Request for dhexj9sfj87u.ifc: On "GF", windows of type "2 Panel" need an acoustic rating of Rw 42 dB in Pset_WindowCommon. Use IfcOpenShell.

First a look at what the model holds.

```python
import ifcopenshell
import ifcopenshell.util.element

model = ifcopenshell.open("dhexj9sfj87u.ifc")
print(model.schema)
storey = next(s for s in model.by_type("IfcBuildingStorey") if s.Name == "GF")
windows = [e for e in ifcopenshell.util.element.get_decomposition(storey) if e.is_a("IfcWindow")]
seen = {}
for e in windows:
    element_type = ifcopenshell.util.element.get_type(e)
    key = (element_type.Name if element_type != e and element_type else None, ifcopenshell.util.element.get_pset(e, "Pset_WindowCommon", "AcousticRating"))
    seen[key] = seen.get(key, 0) + 1
for (name, value), count in sorted(seen.items(), key=str):
    print(count, "x", name, "|", value)
```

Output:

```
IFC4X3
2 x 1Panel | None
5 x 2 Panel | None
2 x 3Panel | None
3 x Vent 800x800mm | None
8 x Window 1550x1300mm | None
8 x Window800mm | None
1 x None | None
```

```python
import ifcopenshell
import ifcopenshell.api.pset
import ifcopenshell.util.element

model = ifcopenshell.open("dhexj9sfj87u.ifc")

storey = next(s for s in model.by_type("IfcBuildingStorey") if s.Name == "GF")
windows = [e for e in ifcopenshell.util.element.get_decomposition(storey) if e.is_a("IfcWindow")]

count = 0
for e in windows:
    element_type = ifcopenshell.util.element.get_type(e)
    if element_type in (None, e) or element_type.Name != "2 Panel":
        continue
    # add_pset returns the element's existing set when there is one.
    pset = ifcopenshell.api.pset.add_pset(model, product=e, name="Pset_WindowCommon")
    ifcopenshell.api.pset.edit_pset(model, pset=pset, properties={"AcousticRating": "Rw 42 dB"})
    count += 1

print(count, "windows updated")

model.write("dhexj9sfj87u_edited.ifc")
```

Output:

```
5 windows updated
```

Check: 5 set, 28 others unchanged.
